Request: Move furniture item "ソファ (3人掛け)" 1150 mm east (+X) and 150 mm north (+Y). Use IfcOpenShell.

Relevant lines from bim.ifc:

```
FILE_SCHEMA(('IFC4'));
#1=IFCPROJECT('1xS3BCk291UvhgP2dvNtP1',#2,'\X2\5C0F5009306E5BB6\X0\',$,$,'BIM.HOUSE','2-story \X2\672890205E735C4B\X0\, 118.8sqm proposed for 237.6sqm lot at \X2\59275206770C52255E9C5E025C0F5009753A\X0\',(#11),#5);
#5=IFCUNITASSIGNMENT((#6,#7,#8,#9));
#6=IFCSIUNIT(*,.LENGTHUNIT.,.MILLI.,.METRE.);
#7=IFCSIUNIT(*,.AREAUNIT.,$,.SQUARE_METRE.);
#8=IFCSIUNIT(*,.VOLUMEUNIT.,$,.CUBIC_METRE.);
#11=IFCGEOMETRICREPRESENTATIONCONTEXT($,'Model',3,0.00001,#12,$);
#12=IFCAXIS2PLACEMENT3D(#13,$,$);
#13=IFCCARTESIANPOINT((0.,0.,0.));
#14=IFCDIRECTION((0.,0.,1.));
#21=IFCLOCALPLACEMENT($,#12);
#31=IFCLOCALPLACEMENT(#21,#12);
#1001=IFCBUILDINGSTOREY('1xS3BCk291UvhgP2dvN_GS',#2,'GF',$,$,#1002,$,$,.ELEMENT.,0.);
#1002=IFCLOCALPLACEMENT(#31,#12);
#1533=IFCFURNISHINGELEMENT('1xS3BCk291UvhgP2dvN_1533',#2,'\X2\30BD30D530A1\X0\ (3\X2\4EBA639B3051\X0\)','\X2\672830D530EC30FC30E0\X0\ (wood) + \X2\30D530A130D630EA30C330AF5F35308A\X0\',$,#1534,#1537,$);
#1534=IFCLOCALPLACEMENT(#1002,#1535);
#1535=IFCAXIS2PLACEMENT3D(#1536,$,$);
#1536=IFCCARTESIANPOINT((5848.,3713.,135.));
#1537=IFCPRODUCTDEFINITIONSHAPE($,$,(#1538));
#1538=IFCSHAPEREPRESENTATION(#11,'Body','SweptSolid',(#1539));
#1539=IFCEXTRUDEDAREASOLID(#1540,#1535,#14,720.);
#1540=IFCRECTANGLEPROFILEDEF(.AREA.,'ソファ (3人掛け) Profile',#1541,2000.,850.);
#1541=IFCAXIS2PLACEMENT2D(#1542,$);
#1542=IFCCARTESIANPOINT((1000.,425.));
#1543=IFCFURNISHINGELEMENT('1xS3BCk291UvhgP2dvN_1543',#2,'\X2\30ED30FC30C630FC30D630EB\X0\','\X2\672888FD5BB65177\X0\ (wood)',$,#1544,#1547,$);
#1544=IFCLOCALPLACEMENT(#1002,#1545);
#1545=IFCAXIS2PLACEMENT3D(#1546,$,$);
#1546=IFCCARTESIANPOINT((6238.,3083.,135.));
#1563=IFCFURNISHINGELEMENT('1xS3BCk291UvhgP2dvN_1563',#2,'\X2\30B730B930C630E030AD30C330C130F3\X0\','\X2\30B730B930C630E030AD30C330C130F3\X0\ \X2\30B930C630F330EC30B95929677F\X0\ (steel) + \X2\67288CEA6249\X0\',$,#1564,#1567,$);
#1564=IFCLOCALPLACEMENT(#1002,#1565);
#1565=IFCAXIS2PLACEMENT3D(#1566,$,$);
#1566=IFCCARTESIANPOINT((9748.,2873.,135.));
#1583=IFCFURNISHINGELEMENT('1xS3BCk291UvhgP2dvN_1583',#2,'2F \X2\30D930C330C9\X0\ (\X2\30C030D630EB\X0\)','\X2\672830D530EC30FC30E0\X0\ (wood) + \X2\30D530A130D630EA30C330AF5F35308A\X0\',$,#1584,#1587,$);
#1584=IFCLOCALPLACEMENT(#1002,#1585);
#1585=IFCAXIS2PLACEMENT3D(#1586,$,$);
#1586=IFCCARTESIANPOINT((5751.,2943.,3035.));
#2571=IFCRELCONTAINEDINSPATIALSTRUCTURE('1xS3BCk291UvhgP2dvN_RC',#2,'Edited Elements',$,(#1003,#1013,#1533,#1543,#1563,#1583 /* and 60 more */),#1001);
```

```python
import ifcopenshell
import ifcopenshell.api.geometry
import ifcopenshell.util.placement

model = ifcopenshell.open("bim.ifc")

item = model.by_id(1533)
matrix = ifcopenshell.util.placement.get_local_placement(item.ObjectPlacement)
matrix[0, 3] += 1150.0
matrix[1, 3] += 150.0
ifcopenshell.api.geometry.edit_object_placement(model, product=item, matrix=matrix, is_si=False)

print(ifcopenshell.util.placement.get_local_placement(item.ObjectPlacement).round(3) + 0.0)

model.write("bim_rev.ifc")
```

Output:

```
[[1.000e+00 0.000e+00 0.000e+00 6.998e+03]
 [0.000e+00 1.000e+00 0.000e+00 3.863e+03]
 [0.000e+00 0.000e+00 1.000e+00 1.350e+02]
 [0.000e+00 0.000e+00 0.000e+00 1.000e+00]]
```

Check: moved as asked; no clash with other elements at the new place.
